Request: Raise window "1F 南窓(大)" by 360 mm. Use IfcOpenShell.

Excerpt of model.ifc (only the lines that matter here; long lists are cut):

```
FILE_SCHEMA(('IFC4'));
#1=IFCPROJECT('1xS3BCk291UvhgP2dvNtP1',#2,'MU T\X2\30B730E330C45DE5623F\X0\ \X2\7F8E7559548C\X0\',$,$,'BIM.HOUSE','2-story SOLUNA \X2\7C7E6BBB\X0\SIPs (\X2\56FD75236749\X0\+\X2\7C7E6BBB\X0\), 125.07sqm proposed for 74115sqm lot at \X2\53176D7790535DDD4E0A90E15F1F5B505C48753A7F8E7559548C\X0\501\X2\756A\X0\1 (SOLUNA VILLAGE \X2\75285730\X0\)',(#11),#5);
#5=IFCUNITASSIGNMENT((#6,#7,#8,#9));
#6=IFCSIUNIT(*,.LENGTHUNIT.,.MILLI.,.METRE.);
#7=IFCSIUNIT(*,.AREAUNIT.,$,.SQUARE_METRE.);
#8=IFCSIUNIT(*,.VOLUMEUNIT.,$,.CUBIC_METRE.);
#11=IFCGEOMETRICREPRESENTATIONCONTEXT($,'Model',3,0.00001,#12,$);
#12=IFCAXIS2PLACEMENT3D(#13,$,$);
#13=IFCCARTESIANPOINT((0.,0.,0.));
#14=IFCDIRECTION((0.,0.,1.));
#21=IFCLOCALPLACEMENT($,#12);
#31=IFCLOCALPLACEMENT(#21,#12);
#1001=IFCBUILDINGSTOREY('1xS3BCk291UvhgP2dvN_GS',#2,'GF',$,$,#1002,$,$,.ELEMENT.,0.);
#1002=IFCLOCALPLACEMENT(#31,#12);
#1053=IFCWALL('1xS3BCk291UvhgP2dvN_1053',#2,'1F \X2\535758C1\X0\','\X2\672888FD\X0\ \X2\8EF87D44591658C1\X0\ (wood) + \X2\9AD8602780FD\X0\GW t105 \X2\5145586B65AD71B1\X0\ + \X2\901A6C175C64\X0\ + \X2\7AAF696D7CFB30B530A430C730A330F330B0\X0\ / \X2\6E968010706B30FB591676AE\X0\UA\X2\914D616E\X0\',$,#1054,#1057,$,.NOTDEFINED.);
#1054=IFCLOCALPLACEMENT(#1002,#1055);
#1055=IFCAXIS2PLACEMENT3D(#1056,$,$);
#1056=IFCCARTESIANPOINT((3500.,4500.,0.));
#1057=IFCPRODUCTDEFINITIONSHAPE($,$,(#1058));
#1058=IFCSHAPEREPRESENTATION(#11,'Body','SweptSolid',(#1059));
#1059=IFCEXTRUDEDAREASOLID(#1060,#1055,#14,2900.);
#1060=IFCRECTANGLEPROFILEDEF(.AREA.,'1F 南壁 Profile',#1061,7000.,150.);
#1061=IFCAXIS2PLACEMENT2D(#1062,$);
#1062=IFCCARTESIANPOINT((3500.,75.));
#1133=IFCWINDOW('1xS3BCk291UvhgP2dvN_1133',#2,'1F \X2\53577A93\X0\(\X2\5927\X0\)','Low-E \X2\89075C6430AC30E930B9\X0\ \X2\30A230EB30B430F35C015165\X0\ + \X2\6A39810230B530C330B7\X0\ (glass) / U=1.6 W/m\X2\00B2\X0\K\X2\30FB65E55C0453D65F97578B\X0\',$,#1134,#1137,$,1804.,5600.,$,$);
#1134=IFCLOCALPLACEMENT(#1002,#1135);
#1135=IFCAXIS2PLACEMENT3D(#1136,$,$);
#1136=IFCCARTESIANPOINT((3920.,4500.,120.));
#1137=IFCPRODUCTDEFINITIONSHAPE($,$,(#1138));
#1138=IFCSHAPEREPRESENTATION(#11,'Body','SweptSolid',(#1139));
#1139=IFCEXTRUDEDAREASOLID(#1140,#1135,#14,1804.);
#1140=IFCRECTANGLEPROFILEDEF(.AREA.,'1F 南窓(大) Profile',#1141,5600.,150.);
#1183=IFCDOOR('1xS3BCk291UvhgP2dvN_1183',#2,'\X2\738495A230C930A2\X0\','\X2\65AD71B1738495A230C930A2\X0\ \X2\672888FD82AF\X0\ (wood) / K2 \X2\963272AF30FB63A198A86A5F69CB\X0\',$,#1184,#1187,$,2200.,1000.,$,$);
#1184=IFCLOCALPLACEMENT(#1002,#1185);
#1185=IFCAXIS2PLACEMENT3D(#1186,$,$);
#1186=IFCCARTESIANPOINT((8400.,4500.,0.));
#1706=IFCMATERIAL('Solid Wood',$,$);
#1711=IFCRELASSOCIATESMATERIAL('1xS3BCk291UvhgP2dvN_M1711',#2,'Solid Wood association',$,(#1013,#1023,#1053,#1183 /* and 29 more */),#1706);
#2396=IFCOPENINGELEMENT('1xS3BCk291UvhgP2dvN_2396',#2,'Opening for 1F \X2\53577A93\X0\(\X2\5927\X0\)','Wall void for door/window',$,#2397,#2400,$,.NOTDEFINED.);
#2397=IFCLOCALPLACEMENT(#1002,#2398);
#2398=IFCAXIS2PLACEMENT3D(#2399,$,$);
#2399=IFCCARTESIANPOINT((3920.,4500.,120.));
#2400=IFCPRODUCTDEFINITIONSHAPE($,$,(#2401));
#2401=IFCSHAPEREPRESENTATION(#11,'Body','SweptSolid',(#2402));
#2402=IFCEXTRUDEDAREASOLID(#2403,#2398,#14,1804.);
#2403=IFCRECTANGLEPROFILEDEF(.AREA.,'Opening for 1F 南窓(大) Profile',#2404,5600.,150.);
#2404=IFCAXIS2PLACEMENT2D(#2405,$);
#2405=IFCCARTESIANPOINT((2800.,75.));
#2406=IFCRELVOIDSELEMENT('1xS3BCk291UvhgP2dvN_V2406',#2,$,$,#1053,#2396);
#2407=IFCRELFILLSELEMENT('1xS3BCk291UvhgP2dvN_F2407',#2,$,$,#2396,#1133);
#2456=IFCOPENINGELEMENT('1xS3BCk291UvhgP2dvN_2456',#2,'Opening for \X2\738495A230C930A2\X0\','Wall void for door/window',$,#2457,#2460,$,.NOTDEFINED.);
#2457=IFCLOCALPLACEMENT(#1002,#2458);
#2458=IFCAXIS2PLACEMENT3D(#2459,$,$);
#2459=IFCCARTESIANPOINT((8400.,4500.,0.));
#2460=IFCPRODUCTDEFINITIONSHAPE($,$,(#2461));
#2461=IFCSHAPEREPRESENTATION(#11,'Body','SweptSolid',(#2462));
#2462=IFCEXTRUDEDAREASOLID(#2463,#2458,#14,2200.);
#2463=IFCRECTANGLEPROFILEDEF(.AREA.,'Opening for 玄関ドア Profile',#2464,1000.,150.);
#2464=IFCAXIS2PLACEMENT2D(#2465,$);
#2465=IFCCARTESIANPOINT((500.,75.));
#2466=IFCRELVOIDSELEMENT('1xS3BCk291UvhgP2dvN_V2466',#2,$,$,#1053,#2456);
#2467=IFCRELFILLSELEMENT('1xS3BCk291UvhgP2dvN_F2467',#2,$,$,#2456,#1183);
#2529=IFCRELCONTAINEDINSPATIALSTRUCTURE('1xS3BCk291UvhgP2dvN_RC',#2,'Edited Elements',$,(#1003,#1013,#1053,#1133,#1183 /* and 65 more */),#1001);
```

```python
import numpy as np
import ifcopenshell
import ifcopenshell.api.geometry
import ifcopenshell.util.placement
import ifcopenshell.util.unit

model = ifcopenshell.open("model.ifc")
unit_scale = ifcopenshell.util.unit.calculate_unit_scale(model)

window = model.by_guid("1xS3BCk291UvhgP2dvN_1133")
opening = window.FillsVoids[0].RelatingOpeningElement
dz = 360.0

shift = np.array([0.0, 0.0, dz])
# The window is not placed relative to its opening, so move both.
for product in (opening, window):
    matrix = ifcopenshell.util.placement.get_local_placement(product.ObjectPlacement)
    matrix[:3, 3] += shift
    ifcopenshell.api.geometry.edit_object_placement(model, product=product, matrix=matrix, is_si=False)

print(f"moved by {dz * unit_scale:+.3f} m")

model.write("model_updated.ifc")
```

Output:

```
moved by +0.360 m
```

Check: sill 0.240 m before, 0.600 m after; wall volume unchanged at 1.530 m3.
